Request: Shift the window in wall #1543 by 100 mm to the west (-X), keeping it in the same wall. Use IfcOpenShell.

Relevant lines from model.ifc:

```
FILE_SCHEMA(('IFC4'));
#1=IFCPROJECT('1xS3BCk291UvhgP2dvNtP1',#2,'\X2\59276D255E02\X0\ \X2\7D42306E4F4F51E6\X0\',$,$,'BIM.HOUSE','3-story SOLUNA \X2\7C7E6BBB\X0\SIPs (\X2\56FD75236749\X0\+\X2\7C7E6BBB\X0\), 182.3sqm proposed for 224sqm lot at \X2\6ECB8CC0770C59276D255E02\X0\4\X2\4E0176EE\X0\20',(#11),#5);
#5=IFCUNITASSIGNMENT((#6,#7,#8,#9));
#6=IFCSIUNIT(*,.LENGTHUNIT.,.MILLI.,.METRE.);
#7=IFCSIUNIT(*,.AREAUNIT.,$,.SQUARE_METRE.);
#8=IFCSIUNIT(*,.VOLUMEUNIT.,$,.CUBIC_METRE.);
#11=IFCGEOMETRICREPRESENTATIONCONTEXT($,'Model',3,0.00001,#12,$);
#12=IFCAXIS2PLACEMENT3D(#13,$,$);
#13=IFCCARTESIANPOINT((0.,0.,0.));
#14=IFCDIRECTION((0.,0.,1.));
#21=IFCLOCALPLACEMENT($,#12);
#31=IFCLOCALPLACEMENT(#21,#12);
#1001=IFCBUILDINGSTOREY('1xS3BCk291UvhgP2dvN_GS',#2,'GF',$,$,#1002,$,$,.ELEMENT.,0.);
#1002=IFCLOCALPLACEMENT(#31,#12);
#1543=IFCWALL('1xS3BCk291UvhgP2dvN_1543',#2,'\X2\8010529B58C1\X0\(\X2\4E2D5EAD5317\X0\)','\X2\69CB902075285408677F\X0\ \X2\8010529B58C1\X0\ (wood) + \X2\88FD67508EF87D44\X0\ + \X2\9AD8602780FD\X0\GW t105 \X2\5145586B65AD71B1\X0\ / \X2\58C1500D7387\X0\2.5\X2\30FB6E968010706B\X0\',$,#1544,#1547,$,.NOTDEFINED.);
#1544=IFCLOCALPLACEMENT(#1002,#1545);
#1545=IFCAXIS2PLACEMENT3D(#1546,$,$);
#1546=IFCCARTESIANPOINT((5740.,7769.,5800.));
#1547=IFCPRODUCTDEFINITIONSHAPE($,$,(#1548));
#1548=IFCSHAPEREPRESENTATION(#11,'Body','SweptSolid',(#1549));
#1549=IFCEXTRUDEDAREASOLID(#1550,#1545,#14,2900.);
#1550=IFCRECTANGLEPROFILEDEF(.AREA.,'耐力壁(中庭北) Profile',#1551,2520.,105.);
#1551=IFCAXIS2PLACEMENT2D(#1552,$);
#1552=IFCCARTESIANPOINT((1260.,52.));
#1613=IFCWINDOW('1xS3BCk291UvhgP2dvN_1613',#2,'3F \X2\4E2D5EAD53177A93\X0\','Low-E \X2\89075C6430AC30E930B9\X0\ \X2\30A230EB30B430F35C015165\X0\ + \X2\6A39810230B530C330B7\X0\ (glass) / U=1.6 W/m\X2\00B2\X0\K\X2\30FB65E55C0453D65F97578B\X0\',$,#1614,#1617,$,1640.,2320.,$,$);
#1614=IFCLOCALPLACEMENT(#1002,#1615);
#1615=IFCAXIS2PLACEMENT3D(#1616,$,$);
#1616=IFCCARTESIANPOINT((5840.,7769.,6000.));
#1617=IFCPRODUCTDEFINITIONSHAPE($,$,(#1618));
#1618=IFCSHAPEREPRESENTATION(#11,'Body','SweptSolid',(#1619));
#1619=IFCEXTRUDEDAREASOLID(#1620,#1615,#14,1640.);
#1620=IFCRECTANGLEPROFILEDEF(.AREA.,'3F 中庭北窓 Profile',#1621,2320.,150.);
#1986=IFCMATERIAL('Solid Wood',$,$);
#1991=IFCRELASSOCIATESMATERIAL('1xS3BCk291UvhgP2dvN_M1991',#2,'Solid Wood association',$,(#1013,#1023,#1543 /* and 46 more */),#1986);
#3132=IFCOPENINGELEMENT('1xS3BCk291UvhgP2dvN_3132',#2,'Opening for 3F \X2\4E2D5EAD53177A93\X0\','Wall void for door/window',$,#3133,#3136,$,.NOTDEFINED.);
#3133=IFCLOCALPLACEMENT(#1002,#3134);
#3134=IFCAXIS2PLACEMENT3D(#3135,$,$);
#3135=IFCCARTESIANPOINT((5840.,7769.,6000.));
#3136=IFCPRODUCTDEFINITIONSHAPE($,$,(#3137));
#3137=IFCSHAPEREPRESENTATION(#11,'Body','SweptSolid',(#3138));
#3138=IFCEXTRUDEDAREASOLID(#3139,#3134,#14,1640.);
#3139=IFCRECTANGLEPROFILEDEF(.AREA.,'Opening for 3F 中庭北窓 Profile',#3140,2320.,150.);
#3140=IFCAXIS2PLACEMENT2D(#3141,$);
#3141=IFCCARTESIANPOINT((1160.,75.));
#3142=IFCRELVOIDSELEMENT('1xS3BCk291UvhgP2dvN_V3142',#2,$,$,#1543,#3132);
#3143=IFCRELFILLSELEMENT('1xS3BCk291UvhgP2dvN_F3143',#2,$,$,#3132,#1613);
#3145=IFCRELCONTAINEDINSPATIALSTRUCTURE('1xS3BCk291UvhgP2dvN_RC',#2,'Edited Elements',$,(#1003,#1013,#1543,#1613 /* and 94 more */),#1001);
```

```python
import ifcopenshell
import ifcopenshell.api.geometry
import ifcopenshell.util.placement
import ifcopenshell.util.unit

model = ifcopenshell.open("model.ifc")
unit_scale = ifcopenshell.util.unit.calculate_unit_scale(model)

window = model.by_guid("1xS3BCk291UvhgP2dvN_1613")
opening = window.FillsVoids[0].RelatingOpeningElement
wall = opening.VoidsElements[0].RelatingBuildingElement

wall_matrix = ifcopenshell.util.placement.get_local_placement(wall.ObjectPlacement)
shift = wall_matrix[:3, 0] * -0.1 / unit_scale
before = ifcopenshell.util.placement.get_local_placement(window.ObjectPlacement)[:3, 3].copy()

# The window is not placed relative to its opening, so move both.
for product in (opening, window):
    matrix = ifcopenshell.util.placement.get_local_placement(product.ObjectPlacement)
    matrix[:3, 3] += shift
    ifcopenshell.api.geometry.edit_object_placement(model, product=product, matrix=matrix, is_si=False)

after = ifcopenshell.util.placement.get_local_placement(window.ObjectPlacement)[:3, 3]
print("window moved by", (after - before).round(3) + 0.0)

model.write("model_v2.ifc")
```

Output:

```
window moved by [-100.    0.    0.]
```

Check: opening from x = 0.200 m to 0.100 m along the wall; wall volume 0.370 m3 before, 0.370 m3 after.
